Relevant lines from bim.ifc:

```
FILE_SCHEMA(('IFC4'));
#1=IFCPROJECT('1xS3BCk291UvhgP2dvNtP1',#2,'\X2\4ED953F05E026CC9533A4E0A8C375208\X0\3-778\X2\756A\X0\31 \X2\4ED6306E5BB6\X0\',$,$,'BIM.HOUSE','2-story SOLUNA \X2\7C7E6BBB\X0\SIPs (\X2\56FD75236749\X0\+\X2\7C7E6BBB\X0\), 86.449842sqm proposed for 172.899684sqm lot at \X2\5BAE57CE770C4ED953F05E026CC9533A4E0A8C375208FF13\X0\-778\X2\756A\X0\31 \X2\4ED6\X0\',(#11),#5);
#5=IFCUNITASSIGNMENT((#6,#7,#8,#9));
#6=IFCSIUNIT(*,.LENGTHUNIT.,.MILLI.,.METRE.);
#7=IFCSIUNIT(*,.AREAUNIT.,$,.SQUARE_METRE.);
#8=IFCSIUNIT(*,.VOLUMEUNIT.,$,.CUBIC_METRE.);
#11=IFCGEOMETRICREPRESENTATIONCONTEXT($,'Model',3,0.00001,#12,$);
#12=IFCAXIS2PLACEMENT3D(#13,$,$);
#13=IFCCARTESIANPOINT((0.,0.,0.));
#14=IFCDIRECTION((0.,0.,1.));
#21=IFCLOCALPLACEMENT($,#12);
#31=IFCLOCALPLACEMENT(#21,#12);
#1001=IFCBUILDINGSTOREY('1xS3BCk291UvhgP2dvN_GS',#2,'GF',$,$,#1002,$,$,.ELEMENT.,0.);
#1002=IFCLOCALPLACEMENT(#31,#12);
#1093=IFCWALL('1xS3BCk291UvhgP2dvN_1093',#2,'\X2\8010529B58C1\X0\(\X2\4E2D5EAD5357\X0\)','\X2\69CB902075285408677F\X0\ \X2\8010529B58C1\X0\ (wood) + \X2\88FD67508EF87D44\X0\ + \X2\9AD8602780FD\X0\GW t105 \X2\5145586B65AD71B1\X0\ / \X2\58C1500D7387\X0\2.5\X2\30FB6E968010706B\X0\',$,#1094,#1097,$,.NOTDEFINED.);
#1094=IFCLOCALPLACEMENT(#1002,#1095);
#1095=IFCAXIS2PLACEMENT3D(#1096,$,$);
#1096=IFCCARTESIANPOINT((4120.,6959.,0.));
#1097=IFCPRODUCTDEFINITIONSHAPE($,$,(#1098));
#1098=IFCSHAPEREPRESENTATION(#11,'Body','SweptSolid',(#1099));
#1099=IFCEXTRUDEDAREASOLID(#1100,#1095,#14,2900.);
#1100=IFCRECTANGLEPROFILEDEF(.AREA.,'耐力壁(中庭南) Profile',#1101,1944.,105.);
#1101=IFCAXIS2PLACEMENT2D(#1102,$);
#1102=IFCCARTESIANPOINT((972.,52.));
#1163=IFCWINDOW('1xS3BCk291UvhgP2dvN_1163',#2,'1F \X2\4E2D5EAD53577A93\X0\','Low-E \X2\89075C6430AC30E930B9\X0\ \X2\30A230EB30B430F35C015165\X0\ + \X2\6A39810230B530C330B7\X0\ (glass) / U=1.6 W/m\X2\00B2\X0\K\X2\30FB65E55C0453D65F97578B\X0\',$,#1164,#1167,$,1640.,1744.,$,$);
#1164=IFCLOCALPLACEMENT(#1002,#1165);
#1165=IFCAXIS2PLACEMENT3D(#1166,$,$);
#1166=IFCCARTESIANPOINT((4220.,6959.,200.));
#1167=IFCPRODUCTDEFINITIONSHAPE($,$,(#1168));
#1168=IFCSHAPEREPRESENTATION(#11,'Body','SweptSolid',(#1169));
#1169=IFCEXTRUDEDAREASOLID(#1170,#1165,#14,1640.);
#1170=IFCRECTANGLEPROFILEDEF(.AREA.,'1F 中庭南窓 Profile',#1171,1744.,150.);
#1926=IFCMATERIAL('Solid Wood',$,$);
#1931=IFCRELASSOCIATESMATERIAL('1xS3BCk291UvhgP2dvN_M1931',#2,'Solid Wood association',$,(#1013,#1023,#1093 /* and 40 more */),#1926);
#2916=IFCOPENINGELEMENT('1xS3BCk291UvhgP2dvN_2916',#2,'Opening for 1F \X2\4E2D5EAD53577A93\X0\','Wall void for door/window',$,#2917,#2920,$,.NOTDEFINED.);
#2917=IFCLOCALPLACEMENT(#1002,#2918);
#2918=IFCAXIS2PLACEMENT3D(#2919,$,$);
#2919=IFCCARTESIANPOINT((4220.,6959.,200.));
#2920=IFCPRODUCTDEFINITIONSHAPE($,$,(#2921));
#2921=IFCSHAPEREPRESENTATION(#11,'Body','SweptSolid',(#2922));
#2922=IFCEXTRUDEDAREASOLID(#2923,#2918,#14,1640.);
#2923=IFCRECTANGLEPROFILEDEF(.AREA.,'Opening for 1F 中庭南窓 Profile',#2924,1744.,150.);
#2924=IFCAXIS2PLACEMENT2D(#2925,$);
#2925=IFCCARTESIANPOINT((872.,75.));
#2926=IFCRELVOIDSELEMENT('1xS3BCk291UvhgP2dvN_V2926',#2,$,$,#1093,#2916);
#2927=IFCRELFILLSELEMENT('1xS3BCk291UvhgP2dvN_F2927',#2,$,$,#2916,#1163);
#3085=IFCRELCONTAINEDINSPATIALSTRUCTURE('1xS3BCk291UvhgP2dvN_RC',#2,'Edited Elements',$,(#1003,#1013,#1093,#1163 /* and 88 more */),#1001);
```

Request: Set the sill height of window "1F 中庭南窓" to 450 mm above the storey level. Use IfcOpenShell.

```python
import numpy as np
import ifcopenshell
import ifcopenshell.api.geometry
import ifcopenshell.geom
import ifcopenshell.util.element
import ifcopenshell.util.placement
import ifcopenshell.util.shape
import ifcopenshell.util.unit

model = ifcopenshell.open("bim.ifc")
unit_scale = ifcopenshell.util.unit.calculate_unit_scale(model)

window = model.by_guid("1xS3BCk291UvhgP2dvN_1163")
opening = window.FillsVoids[0].RelatingOpeningElement
storey = ifcopenshell.util.element.get_container(window, ifc_class="IfcBuildingStorey")
level = ifcopenshell.util.placement.get_local_placement(storey.ObjectPlacement)[2, 3]

# The opening's origin need not be at the sill, so measure its lowest point.
shape = ifcopenshell.geom.create_shape(ifcopenshell.geom.settings(), opening)
bottom = ifcopenshell.util.shape.get_shape_bottom_elevation(shape, shape.geometry) / unit_scale
dz = level + 0.45 / unit_scale - bottom

shift = np.array([0.0, 0.0, dz])
# The window is not placed relative to its opening, so move both.
for product in (opening, window):
    matrix = ifcopenshell.util.placement.get_local_placement(product.ObjectPlacement)
    matrix[:3, 3] += shift
    ifcopenshell.api.geometry.edit_object_placement(model, product=product, matrix=matrix, is_si=False)

print(f"moved by {dz * unit_scale:+.3f} m")

model.write("bim-out.ifc")
```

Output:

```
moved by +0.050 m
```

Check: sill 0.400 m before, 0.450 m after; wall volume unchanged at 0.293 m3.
